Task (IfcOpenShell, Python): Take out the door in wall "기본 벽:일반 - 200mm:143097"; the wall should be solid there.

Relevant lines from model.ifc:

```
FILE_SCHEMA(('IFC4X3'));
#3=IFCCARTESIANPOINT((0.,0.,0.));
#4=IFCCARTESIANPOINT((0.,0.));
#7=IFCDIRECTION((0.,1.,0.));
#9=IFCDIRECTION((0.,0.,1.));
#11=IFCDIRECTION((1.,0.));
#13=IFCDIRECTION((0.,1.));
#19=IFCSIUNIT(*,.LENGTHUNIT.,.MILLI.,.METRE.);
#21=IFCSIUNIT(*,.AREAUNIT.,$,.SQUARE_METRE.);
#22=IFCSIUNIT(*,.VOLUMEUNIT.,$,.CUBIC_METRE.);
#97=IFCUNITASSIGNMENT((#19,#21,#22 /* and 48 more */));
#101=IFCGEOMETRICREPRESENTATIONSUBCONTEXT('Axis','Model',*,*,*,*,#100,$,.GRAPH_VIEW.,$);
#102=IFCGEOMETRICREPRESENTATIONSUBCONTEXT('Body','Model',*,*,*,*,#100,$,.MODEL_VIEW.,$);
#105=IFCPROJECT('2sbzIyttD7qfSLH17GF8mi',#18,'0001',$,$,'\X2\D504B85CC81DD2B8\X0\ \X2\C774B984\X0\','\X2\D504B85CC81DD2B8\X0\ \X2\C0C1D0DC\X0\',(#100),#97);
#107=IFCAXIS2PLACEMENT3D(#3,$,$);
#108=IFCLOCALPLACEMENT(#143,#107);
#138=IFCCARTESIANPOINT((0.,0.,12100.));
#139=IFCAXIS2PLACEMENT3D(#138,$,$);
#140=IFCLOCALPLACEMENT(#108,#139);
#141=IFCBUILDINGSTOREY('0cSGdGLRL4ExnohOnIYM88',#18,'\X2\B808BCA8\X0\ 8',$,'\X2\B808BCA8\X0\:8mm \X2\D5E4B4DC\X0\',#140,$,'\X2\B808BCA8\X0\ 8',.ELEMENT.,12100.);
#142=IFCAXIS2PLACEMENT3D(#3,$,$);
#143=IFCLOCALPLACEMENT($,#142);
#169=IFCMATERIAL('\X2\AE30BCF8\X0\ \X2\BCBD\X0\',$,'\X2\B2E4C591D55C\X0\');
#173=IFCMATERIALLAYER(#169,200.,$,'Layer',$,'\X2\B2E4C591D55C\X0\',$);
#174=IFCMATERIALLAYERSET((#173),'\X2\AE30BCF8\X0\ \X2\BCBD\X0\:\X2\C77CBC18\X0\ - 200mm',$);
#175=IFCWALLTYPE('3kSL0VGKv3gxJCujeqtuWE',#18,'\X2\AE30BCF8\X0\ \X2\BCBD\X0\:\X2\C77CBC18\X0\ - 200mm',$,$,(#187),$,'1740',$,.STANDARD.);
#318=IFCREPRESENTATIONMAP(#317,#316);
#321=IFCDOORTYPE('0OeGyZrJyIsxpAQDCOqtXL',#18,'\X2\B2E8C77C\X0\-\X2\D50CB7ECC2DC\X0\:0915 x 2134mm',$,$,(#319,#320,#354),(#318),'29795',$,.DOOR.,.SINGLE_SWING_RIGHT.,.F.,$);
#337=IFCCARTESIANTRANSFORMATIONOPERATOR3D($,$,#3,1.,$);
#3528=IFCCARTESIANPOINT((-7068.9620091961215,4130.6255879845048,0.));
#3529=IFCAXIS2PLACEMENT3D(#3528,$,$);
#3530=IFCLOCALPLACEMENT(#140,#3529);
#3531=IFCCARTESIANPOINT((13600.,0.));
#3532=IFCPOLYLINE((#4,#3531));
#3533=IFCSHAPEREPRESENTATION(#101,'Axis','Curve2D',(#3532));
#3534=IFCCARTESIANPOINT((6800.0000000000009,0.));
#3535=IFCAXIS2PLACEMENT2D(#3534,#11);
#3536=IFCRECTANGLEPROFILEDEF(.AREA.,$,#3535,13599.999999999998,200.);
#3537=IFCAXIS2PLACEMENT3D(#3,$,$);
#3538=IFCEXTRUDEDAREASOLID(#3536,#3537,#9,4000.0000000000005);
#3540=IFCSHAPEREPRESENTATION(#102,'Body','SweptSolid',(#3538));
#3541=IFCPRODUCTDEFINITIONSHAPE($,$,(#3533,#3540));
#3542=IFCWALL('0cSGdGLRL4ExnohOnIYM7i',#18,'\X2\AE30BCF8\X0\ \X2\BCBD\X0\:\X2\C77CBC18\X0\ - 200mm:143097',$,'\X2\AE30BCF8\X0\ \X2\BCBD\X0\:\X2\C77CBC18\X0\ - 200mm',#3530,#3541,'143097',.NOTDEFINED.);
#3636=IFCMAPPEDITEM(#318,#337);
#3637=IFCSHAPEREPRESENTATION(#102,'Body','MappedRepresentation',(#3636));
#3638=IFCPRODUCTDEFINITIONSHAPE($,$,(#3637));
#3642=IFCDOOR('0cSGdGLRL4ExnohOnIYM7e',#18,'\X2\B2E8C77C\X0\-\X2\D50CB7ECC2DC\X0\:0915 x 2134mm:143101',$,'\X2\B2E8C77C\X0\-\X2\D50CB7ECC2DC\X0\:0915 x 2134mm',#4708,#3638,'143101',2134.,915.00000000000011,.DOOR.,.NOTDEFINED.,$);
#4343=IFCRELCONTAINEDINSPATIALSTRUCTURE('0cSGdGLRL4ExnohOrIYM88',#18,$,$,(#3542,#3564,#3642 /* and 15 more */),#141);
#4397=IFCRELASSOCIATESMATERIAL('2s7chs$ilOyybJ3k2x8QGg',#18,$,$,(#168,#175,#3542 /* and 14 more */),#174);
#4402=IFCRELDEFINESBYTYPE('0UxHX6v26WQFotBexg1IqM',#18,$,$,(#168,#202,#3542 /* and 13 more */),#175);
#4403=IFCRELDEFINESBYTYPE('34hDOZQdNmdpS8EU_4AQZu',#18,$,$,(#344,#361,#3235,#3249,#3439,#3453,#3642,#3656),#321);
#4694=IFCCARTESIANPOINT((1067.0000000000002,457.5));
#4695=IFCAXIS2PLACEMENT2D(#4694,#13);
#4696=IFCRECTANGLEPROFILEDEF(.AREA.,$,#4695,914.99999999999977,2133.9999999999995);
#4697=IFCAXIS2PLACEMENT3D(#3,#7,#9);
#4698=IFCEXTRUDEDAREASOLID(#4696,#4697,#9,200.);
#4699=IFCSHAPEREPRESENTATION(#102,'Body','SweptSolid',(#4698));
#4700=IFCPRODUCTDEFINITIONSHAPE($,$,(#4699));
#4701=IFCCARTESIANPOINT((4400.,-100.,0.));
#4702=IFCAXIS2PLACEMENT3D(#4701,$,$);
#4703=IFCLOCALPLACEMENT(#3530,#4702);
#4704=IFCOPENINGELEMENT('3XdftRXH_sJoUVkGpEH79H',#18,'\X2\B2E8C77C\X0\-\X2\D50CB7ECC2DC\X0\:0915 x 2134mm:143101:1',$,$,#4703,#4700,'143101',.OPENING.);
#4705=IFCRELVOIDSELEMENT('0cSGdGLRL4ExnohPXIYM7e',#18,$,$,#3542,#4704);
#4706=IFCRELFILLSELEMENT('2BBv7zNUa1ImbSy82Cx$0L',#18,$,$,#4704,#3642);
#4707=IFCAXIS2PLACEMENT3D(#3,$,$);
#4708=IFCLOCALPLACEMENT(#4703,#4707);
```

```python
import ifcopenshell
import ifcopenshell.api.feature
import ifcopenshell.api.root
import ifcopenshell.geom
import ifcopenshell.util.shape

model = ifcopenshell.open("model.ifc")
settings = ifcopenshell.geom.settings()


def volume(element):
    """Net volume in cubic metres, openings subtracted."""
    shape = ifcopenshell.geom.create_shape(settings, element)
    return ifcopenshell.util.shape.get_volume(shape.geometry)


door = model.by_guid("0cSGdGLRL4ExnohOnIYM7e")
opening = door.FillsVoids[0].RelatingOpeningElement
wall = opening.VoidsElements[0].RelatingBuildingElement
before = volume(wall)

ifcopenshell.api.root.remove_product(model, product=door)
ifcopenshell.api.feature.remove_feature(model, feature=opening)

after = volume(wall)

print(f"wall volume {before:.3f} -> {after:.3f} m3")

model.write("model-out.ifc")
```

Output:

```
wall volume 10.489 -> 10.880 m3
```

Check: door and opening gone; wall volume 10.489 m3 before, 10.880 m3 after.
